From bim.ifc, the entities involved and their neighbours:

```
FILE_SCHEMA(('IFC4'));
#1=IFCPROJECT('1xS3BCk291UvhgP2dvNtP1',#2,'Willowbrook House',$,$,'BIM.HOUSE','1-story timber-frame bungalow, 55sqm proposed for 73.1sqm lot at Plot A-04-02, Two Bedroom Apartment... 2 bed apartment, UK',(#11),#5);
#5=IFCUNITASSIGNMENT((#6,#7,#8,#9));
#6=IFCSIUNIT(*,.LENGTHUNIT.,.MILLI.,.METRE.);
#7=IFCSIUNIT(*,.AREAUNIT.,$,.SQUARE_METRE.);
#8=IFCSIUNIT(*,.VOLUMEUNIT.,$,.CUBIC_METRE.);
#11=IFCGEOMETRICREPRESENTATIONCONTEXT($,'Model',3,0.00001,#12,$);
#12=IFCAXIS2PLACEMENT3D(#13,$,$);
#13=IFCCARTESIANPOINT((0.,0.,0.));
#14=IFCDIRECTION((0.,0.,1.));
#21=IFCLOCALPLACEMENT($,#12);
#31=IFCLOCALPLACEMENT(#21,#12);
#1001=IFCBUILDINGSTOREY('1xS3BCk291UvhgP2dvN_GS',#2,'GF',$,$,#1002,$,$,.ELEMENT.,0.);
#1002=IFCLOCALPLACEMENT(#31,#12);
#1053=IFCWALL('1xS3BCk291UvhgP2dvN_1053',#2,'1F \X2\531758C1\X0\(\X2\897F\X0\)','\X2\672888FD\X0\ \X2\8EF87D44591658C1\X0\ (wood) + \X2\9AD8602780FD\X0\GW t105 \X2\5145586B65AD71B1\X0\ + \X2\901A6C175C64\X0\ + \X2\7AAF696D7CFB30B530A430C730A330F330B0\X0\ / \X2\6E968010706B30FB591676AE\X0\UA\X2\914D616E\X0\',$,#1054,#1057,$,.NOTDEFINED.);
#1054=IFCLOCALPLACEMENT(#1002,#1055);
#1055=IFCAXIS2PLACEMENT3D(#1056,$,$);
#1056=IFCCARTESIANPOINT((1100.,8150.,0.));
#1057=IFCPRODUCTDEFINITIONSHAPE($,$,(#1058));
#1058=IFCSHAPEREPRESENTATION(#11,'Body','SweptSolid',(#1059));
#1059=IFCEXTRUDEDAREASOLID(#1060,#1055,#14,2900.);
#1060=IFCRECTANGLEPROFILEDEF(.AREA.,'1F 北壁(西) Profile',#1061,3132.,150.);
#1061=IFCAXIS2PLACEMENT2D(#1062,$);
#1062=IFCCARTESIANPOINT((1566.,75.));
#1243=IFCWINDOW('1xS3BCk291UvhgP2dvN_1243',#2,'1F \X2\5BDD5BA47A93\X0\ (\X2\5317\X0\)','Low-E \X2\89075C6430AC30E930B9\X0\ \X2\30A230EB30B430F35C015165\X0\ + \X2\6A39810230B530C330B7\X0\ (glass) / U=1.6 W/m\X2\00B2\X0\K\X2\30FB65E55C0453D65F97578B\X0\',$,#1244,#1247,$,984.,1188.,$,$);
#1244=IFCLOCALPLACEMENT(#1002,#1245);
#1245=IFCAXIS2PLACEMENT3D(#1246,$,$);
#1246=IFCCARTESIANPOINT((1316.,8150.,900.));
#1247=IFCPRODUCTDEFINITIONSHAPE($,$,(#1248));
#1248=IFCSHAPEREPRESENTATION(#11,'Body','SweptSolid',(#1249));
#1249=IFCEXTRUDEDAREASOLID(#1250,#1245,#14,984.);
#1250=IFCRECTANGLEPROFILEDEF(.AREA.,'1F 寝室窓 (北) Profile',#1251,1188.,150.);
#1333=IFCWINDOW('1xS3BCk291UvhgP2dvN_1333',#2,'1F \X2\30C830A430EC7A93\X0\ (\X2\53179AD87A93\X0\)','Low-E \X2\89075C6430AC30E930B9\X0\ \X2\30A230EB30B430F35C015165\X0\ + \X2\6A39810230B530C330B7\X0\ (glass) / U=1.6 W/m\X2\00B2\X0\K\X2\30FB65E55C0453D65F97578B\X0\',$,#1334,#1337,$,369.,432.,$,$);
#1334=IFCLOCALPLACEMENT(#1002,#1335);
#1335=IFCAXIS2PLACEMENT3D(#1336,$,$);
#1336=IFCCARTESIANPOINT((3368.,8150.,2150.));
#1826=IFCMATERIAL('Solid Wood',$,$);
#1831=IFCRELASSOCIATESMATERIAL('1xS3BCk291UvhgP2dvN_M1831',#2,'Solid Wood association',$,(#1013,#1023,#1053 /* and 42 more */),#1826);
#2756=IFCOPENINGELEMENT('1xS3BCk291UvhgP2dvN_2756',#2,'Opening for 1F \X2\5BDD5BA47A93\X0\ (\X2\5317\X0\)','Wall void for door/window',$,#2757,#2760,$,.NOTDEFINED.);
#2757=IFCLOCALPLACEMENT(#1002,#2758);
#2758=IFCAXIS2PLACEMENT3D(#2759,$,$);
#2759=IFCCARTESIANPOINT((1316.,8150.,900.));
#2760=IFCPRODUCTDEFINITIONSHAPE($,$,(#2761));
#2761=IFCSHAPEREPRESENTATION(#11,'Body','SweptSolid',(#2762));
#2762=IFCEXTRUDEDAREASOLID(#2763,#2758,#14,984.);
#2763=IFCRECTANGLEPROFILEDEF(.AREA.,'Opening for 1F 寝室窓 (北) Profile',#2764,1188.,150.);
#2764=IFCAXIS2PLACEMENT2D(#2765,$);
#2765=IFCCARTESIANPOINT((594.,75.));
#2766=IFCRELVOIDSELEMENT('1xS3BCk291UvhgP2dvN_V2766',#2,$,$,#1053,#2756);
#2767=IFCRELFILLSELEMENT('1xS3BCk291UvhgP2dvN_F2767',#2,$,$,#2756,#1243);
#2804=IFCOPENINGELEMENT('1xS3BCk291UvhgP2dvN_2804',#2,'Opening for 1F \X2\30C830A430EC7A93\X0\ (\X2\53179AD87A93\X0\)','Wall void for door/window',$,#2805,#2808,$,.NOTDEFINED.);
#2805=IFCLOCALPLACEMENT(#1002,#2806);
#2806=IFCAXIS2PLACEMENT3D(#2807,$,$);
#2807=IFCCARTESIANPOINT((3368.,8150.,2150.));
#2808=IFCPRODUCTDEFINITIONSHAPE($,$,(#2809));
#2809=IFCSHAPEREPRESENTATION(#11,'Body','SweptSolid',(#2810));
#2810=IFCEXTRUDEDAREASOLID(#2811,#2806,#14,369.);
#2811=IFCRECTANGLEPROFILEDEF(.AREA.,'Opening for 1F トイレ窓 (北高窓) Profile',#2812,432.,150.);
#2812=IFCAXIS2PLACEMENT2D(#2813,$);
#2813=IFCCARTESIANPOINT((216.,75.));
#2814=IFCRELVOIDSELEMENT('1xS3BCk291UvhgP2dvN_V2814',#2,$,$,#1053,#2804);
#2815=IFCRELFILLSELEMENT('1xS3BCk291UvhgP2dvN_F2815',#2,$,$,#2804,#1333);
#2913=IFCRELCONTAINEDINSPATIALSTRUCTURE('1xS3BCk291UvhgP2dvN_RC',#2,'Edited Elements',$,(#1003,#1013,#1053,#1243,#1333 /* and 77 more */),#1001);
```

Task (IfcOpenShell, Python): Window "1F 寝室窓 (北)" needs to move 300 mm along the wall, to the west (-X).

```python
import ifcopenshell
import ifcopenshell.api.geometry
import ifcopenshell.util.placement
import ifcopenshell.util.unit

model = ifcopenshell.open("bim.ifc")
unit_scale = ifcopenshell.util.unit.calculate_unit_scale(model)

window = model.by_id(1243)
opening = window.FillsVoids[0].RelatingOpeningElement
wall = opening.VoidsElements[0].RelatingBuildingElement

wall_matrix = ifcopenshell.util.placement.get_local_placement(wall.ObjectPlacement)
shift = wall_matrix[:3, 0] * -0.3 / unit_scale
before = ifcopenshell.util.placement.get_local_placement(window.ObjectPlacement)[:3, 3].copy()

# The window is not placed relative to its opening, so move both.
for product in (opening, window):
    matrix = ifcopenshell.util.placement.get_local_placement(product.ObjectPlacement)
    matrix[:3, 3] += shift
    ifcopenshell.api.geometry.edit_object_placement(model, product=product, matrix=matrix, is_si=False)

after = ifcopenshell.util.placement.get_local_placement(window.ObjectPlacement)[:3, 3]
print("window moved by", (after - before).round(3) + 0.0)

model.write("bim-out.ifc")
```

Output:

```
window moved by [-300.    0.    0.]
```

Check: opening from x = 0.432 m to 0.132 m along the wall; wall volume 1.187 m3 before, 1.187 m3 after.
